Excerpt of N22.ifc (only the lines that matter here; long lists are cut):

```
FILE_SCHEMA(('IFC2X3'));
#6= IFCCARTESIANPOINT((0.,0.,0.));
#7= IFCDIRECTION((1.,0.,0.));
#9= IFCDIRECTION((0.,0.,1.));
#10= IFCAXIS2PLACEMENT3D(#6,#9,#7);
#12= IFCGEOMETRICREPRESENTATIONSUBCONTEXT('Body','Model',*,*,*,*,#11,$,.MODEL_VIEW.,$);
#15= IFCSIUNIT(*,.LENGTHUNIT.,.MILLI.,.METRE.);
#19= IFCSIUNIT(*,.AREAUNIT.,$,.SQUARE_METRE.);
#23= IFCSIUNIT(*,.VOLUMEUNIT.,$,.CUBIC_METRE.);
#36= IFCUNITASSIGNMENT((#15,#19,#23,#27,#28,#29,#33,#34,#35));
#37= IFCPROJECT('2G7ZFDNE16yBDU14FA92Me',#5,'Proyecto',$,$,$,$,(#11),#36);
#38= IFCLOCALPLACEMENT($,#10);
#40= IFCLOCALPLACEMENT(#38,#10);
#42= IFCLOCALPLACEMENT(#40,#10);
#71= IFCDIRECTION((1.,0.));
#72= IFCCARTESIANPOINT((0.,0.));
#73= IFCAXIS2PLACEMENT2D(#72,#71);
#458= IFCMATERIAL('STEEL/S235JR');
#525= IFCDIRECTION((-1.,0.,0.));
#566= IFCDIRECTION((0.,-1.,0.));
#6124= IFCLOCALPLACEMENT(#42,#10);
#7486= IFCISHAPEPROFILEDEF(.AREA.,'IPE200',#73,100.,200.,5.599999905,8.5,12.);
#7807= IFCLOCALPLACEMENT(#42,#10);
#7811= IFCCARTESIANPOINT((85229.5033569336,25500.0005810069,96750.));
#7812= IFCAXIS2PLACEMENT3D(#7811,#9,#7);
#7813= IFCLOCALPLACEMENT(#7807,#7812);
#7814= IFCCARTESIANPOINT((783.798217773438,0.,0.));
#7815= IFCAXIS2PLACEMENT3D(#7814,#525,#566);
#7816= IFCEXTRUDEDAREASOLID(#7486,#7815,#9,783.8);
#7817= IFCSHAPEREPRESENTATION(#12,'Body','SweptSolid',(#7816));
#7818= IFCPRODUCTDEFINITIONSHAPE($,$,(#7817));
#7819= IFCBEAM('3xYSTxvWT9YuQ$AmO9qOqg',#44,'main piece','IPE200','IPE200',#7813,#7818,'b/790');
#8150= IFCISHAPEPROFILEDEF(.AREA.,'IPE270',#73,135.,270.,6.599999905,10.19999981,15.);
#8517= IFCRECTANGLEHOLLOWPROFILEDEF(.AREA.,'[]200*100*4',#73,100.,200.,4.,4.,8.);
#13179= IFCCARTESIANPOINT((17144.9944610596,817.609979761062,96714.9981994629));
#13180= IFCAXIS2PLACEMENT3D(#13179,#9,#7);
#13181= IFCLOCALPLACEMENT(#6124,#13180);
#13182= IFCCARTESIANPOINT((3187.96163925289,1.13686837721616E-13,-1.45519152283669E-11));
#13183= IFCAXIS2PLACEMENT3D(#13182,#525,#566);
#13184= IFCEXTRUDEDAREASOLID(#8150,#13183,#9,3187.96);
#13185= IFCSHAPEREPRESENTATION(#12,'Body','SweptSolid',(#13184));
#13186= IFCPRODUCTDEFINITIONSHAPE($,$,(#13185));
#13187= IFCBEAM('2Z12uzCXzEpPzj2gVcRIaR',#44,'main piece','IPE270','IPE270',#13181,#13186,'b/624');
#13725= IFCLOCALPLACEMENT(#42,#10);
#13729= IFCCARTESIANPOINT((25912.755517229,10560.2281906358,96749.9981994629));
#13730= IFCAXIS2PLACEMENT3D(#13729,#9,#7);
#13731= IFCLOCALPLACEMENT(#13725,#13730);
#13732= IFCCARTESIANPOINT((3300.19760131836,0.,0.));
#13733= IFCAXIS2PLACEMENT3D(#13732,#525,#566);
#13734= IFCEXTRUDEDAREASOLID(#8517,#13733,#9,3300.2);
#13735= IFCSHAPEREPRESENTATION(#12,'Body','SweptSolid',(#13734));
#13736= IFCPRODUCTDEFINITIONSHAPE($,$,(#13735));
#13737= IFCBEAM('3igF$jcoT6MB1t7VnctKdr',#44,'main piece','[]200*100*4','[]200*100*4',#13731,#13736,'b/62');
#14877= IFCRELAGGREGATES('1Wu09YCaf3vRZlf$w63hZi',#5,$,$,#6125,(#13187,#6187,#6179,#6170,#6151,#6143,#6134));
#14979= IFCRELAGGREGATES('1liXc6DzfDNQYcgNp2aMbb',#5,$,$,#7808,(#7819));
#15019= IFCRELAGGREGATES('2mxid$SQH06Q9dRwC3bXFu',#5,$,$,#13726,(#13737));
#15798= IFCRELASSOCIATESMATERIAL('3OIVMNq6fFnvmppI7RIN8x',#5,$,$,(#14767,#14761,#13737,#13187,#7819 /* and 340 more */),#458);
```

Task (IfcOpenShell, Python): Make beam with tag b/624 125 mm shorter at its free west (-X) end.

```python
import ifcopenshell
import ifcopenshell.util.representation
import ifcopenshell.util.unit

model = ifcopenshell.open("N22.ifc")
unit_scale = ifcopenshell.util.unit.calculate_unit_scale(model)

member = model.by_guid("2Z12uzCXzEpPzj2gVcRIaR")
change = -0.125 / unit_scale

# The extrusion runs towards the end named, so only its depth changes.
body = ifcopenshell.util.representation.get_representation(member, "Model", "Body")
solid = body.Items[0]
old_length = solid.Depth
solid.Depth += change

print(f"length {old_length:g} -> {solid.Depth:g}")

model.write("N22_v2.ifc")
```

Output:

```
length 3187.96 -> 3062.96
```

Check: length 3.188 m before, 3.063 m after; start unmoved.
